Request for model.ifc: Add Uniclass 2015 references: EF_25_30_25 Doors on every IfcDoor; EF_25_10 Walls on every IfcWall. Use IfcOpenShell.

First a look at what the model holds.

```python
import ifcopenshell

model = ifcopenshell.open("model.ifc")
print(model.schema)
print("classifications:", [c.Name for c in model.by_type("IfcClassification")])
for ifc_class in ("IfcDoor", "IfcRoof", "IfcStair", "IfcWall", "IfcWindow"):
    print(ifc_class, len(model.by_type(ifc_class)))
```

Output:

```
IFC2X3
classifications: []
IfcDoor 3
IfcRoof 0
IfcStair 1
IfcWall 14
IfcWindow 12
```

```python
import ifcopenshell
import ifcopenshell.api.classification

model = ifcopenshell.open("model.ifc")

# IFC2X3 requires Source and Edition and has no link from the project to the system.
system = model.create_entity("IfcClassification", Source="NBS", Edition="2015", Name="Uniclass 2015")

codes = {
    "IfcDoor": ("EF_25_30_25", "Doors"),
    "IfcWall": ("EF_25_10", "Walls"),
}
for ifc_class, (code, name) in codes.items():
    products = model.by_type(ifc_class)
    ifcopenshell.api.classification.add_reference(
        model, products=products, classification=system, identification=code, name=name
    )
    print(code, len(products))

model.write("model_v2.ifc")
```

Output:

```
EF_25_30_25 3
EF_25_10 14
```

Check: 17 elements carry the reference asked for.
